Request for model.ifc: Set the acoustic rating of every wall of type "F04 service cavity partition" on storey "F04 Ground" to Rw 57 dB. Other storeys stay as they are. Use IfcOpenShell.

First a look at what the model holds.

```python
import ifcopenshell
import ifcopenshell.util.element

model = ifcopenshell.open("model.ifc")
print(model.schema)
storey = next(s for s in model.by_type("IfcBuildingStorey") if s.Name == "F04 Ground")
walls = [e for e in ifcopenshell.util.element.get_decomposition(storey) if e.is_a("IfcWall")]
seen = {}
for e in walls:
    element_type = ifcopenshell.util.element.get_type(e)
    key = (element_type.Name if element_type != e and element_type else None, ifcopenshell.util.element.get_pset(e, "Pset_WallCommon", "AcousticRating"))
    seen[key] = seen.get(key, 0) + 1
for (name, value), count in sorted(seen.items(), key=str):
    print(count, "x", name, "|", value)
```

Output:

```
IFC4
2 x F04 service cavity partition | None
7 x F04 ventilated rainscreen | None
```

```python
import ifcopenshell
import ifcopenshell.api.pset
import ifcopenshell.util.element

model = ifcopenshell.open("model.ifc")

storey = next(s for s in model.by_type("IfcBuildingStorey") if s.Name == "F04 Ground")
walls = [e for e in ifcopenshell.util.element.get_decomposition(storey) if e.is_a("IfcWall")]

count = 0
for e in walls:
    element_type = ifcopenshell.util.element.get_type(e)
    if element_type in (None, e) or element_type.Name != "F04 service cavity partition":
        continue
    # add_pset returns the element's existing set when there is one.
    pset = ifcopenshell.api.pset.add_pset(model, product=e, name="Pset_WallCommon")
    ifcopenshell.api.pset.edit_pset(model, pset=pset, properties={"AcousticRating": "Rw 57 dB"})
    count += 1

print(count, "walls updated")

model.write("model_edited.ifc")
```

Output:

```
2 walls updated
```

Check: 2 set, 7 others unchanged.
